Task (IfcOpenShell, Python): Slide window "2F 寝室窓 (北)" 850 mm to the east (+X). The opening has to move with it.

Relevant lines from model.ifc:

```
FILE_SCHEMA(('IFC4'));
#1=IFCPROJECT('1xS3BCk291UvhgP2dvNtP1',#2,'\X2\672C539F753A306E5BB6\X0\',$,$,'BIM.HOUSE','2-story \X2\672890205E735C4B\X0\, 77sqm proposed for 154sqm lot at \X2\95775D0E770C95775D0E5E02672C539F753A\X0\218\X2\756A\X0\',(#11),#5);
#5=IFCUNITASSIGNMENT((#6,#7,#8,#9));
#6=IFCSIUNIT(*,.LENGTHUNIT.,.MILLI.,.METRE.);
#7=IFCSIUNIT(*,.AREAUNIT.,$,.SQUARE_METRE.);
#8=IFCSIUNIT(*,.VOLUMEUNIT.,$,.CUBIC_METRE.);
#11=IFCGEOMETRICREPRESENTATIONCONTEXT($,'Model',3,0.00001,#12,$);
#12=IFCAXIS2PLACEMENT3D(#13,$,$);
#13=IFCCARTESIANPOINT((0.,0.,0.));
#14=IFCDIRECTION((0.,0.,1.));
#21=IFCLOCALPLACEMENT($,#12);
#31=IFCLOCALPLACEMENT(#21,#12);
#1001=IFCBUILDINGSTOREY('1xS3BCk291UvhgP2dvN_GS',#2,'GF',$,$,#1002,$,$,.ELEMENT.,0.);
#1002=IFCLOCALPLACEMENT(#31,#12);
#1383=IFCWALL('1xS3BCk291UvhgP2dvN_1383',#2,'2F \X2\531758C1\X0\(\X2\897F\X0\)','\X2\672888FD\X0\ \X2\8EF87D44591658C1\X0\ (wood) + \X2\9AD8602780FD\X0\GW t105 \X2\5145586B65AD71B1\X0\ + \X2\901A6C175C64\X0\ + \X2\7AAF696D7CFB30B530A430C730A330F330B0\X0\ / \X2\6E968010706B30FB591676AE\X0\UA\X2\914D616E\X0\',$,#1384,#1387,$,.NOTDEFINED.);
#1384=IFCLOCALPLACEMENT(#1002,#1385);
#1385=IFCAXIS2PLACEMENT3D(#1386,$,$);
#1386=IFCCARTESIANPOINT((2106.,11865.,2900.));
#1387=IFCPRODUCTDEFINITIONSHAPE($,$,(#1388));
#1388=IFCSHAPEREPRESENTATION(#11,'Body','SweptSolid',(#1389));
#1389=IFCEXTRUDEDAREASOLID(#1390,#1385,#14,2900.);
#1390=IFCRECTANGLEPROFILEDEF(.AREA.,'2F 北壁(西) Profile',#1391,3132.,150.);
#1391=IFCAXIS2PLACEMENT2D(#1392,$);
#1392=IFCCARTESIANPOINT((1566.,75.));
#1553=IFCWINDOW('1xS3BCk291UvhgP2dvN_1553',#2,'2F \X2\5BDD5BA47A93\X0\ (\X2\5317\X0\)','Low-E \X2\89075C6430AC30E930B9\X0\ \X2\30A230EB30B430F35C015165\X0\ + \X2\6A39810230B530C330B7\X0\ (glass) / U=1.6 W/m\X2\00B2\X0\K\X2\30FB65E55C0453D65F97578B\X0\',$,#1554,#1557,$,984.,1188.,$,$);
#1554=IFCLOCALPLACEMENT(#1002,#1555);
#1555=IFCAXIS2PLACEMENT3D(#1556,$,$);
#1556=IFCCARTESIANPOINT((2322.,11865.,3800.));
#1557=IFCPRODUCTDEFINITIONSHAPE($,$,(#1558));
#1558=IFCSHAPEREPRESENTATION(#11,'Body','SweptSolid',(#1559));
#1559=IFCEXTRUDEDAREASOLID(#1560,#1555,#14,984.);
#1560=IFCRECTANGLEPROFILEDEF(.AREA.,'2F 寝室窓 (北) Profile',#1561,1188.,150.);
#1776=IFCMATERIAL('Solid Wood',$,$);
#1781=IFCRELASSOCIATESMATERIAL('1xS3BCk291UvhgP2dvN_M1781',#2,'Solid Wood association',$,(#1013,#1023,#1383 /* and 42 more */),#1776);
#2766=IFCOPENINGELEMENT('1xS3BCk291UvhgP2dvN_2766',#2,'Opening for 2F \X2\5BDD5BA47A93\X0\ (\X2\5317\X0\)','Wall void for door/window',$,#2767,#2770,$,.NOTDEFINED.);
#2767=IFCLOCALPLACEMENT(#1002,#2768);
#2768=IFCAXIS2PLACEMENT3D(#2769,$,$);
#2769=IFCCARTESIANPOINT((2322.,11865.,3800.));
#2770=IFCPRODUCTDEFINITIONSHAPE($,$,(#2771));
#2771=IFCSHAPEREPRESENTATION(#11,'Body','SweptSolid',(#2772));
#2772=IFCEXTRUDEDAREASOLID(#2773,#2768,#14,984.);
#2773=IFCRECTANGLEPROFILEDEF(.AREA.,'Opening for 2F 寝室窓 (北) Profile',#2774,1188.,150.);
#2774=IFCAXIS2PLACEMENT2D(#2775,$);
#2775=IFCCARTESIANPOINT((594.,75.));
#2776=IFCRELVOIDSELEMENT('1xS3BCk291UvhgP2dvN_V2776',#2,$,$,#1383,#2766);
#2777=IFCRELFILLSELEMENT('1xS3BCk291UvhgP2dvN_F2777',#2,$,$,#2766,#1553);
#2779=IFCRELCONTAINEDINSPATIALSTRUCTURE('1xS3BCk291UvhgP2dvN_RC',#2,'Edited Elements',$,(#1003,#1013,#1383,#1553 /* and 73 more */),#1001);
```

```python
import ifcopenshell
import ifcopenshell.api.geometry
import ifcopenshell.util.placement
import ifcopenshell.util.unit

model = ifcopenshell.open("model.ifc")
unit_scale = ifcopenshell.util.unit.calculate_unit_scale(model)

window = model.by_guid("1xS3BCk291UvhgP2dvN_1553")
opening = window.FillsVoids[0].RelatingOpeningElement
wall = opening.VoidsElements[0].RelatingBuildingElement

wall_matrix = ifcopenshell.util.placement.get_local_placement(wall.ObjectPlacement)
shift = wall_matrix[:3, 0] * 0.85 / unit_scale
before = ifcopenshell.util.placement.get_local_placement(window.ObjectPlacement)[:3, 3].copy()

# The window is not placed relative to its opening, so move both.
for product in (opening, window):
    matrix = ifcopenshell.util.placement.get_local_placement(product.ObjectPlacement)
    matrix[:3, 3] += shift
    ifcopenshell.api.geometry.edit_object_placement(model, product=product, matrix=matrix, is_si=False)

after = ifcopenshell.util.placement.get_local_placement(window.ObjectPlacement)[:3, 3]
print("window moved by", (after - before).round(3) + 0.0)

model.write("model_v2.ifc")
```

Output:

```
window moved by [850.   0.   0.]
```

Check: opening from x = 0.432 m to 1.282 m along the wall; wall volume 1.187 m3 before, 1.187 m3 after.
